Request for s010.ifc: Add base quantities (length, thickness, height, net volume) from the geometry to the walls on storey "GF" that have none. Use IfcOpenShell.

First a look at what the model holds.

```python
import ifcopenshell
import ifcopenshell.util.element
import ifcopenshell.util.unit

model = ifcopenshell.open("s010.ifc")
print(model.schema)
for unit_type in ("LENGTHUNIT", "AREAUNIT", "VOLUMEUNIT"):
    print(unit_type, ifcopenshell.util.unit.calculate_unit_scale(model, unit_type))
storey = next(s for s in model.by_type("IfcBuildingStorey") if s.Name == "GF")
walls = [e for e in ifcopenshell.util.element.get_decomposition(storey) if e.is_a("IfcWall")]
for e in sorted(walls, key=lambda e: e.id()):
    print(e.id(), e.is_a(), e.Name, list(ifcopenshell.util.element.get_psets(e, qtos_only=True)), sep=" | ")
```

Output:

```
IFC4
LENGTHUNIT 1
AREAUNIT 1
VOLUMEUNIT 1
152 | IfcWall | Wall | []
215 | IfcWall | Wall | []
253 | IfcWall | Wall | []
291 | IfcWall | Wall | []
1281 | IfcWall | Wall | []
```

```python
import ifcopenshell
import ifcopenshell.api.pset
import ifcopenshell.geom
import ifcopenshell.util.element
import ifcopenshell.util.shape
import ifcopenshell.util.unit

model = ifcopenshell.open("s010.ifc")
unit_scale = ifcopenshell.util.unit.calculate_unit_scale(model)
volume_scale = ifcopenshell.util.unit.calculate_unit_scale(model, "VOLUMEUNIT")
settings = ifcopenshell.geom.settings()

storey = next(s for s in model.by_type("IfcBuildingStorey") if s.Name == "GF")
walls = [e for e in ifcopenshell.util.element.get_decomposition(storey) if e.is_a("IfcWall")]

for e in sorted(walls, key=lambda e: e.id()):
    if ifcopenshell.util.element.get_psets(e, qtos_only=True, should_inherit=False):
        continue
    # Geometry comes back in metres, in the element's own axes.
    shape = ifcopenshell.geom.create_shape(settings, e)
    values = {
        "Length": ifcopenshell.util.shape.get_x(shape.geometry) / unit_scale,
        "Width": ifcopenshell.util.shape.get_y(shape.geometry) / unit_scale,
        "Height": ifcopenshell.util.shape.get_z(shape.geometry) / unit_scale,
        "NetVolume": ifcopenshell.util.shape.get_volume(shape.geometry) / volume_scale,
    }
    qto = ifcopenshell.api.pset.add_qto(model, product=e, name="Qto_WallBaseQuantities")
    ifcopenshell.api.pset.edit_qto(model, qto=qto, properties=values)
    print(e.id(), {k: round(v, 3) for k, v in values.items()})

model.write("s010_edited.ifc")
```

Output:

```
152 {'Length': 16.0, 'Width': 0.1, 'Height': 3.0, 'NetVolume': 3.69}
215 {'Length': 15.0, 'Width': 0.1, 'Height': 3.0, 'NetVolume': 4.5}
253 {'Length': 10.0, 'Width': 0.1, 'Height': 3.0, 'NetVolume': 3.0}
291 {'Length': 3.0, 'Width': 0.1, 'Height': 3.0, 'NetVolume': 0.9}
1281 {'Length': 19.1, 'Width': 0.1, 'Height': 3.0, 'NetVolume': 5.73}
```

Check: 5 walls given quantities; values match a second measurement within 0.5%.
